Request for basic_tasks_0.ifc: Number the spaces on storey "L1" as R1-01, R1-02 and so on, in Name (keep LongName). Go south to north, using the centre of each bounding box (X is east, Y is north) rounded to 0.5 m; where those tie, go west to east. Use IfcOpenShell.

First a look at what the model holds.

```python
import ifcopenshell
import ifcopenshell.util.element
import ifcopenshell.util.placement

model = ifcopenshell.open("basic_tasks_0.ifc")
print(model.schema)
storey = next(s for s in model.by_type("IfcBuildingStorey") if s.Name == "L1")
spaces = [e for e in ifcopenshell.util.element.get_decomposition(storey) if e.is_a("IfcSpace")]
for e in sorted(spaces, key=lambda e: e.id()):
    origin = ifcopenshell.util.placement.get_local_placement(e.ObjectPlacement)[:3, 3]
    print(e.id(), e.Name, e.LongName, origin.round(2) + 0.0, sep=" | ")
```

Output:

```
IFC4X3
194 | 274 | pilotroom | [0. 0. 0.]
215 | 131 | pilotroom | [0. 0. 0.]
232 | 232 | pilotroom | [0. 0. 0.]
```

```python
import ifcopenshell
import ifcopenshell.geom
import ifcopenshell.util.element
import ifcopenshell.util.shape

model = ifcopenshell.open("basic_tasks_0.ifc")
settings = ifcopenshell.geom.settings()
settings.set("use-world-coords", True)


def centre(element):
    shape = ifcopenshell.geom.create_shape(settings, element)
    return ifcopenshell.util.shape.get_bbox_centroid(shape.geometry)


storey = next(s for s in model.by_type("IfcBuildingStorey") if s.Name == "L1")
spaces = [e for e in ifcopenshell.util.element.get_decomposition(storey) if e.is_a("IfcSpace")]

# Insertion points can sit at a corner or the storey origin, so sort by the geometry (in metres).
centres = {e: centre(e) for e in spaces}
spaces.sort(key=lambda e: (round(centres[e][1] / 0.5), centres[e][0]))

for i, e in enumerate(spaces, start=1):
    number = f"R1-{i:02d}"
    e.Name = number
    print(e.id(), number)

model.write("basic_tasks_0_updated.ifc")
```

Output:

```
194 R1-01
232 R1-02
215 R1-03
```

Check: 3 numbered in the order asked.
